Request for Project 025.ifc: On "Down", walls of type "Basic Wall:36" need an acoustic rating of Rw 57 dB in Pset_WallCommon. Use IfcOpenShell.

First a look at what the model holds.

```python
import ifcopenshell
import ifcopenshell.util.element

model = ifcopenshell.open("Project 025.ifc")
print(model.schema)
storey = next(s for s in model.by_type("IfcBuildingStorey") if s.Name == "Down")
walls = [e for e in ifcopenshell.util.element.get_decomposition(storey) if e.is_a("IfcWall")]
seen = {}
for e in walls:
    element_type = ifcopenshell.util.element.get_type(e)
    key = (element_type.Name if element_type != e and element_type else None, ifcopenshell.util.element.get_pset(e, "Pset_WallCommon", "AcousticRating"))
    seen[key] = seen.get(key, 0) + 1
for (name, value), count in sorted(seen.items(), key=str):
    print(count, "x", name, "|", value)
```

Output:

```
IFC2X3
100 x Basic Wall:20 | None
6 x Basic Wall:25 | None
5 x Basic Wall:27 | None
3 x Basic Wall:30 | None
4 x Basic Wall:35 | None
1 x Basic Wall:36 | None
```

```python
import ifcopenshell
import ifcopenshell.api.pset
import ifcopenshell.util.element

model = ifcopenshell.open("Project 025.ifc")

storey = next(s for s in model.by_type("IfcBuildingStorey") if s.Name == "Down")
walls = [e for e in ifcopenshell.util.element.get_decomposition(storey) if e.is_a("IfcWall")]

count = 0
for e in walls:
    element_type = ifcopenshell.util.element.get_type(e)
    if element_type in (None, e) or element_type.Name != "Basic Wall:36":
        continue
    # add_pset returns the element's existing set when there is one.
    pset = ifcopenshell.api.pset.add_pset(model, product=e, name="Pset_WallCommon")
    ifcopenshell.api.pset.edit_pset(model, pset=pset, properties={"AcousticRating": "Rw 57 dB"})
    count += 1

print(count, "walls updated")

model.write("Project 025_v2.ifc")
```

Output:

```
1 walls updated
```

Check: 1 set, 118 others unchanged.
